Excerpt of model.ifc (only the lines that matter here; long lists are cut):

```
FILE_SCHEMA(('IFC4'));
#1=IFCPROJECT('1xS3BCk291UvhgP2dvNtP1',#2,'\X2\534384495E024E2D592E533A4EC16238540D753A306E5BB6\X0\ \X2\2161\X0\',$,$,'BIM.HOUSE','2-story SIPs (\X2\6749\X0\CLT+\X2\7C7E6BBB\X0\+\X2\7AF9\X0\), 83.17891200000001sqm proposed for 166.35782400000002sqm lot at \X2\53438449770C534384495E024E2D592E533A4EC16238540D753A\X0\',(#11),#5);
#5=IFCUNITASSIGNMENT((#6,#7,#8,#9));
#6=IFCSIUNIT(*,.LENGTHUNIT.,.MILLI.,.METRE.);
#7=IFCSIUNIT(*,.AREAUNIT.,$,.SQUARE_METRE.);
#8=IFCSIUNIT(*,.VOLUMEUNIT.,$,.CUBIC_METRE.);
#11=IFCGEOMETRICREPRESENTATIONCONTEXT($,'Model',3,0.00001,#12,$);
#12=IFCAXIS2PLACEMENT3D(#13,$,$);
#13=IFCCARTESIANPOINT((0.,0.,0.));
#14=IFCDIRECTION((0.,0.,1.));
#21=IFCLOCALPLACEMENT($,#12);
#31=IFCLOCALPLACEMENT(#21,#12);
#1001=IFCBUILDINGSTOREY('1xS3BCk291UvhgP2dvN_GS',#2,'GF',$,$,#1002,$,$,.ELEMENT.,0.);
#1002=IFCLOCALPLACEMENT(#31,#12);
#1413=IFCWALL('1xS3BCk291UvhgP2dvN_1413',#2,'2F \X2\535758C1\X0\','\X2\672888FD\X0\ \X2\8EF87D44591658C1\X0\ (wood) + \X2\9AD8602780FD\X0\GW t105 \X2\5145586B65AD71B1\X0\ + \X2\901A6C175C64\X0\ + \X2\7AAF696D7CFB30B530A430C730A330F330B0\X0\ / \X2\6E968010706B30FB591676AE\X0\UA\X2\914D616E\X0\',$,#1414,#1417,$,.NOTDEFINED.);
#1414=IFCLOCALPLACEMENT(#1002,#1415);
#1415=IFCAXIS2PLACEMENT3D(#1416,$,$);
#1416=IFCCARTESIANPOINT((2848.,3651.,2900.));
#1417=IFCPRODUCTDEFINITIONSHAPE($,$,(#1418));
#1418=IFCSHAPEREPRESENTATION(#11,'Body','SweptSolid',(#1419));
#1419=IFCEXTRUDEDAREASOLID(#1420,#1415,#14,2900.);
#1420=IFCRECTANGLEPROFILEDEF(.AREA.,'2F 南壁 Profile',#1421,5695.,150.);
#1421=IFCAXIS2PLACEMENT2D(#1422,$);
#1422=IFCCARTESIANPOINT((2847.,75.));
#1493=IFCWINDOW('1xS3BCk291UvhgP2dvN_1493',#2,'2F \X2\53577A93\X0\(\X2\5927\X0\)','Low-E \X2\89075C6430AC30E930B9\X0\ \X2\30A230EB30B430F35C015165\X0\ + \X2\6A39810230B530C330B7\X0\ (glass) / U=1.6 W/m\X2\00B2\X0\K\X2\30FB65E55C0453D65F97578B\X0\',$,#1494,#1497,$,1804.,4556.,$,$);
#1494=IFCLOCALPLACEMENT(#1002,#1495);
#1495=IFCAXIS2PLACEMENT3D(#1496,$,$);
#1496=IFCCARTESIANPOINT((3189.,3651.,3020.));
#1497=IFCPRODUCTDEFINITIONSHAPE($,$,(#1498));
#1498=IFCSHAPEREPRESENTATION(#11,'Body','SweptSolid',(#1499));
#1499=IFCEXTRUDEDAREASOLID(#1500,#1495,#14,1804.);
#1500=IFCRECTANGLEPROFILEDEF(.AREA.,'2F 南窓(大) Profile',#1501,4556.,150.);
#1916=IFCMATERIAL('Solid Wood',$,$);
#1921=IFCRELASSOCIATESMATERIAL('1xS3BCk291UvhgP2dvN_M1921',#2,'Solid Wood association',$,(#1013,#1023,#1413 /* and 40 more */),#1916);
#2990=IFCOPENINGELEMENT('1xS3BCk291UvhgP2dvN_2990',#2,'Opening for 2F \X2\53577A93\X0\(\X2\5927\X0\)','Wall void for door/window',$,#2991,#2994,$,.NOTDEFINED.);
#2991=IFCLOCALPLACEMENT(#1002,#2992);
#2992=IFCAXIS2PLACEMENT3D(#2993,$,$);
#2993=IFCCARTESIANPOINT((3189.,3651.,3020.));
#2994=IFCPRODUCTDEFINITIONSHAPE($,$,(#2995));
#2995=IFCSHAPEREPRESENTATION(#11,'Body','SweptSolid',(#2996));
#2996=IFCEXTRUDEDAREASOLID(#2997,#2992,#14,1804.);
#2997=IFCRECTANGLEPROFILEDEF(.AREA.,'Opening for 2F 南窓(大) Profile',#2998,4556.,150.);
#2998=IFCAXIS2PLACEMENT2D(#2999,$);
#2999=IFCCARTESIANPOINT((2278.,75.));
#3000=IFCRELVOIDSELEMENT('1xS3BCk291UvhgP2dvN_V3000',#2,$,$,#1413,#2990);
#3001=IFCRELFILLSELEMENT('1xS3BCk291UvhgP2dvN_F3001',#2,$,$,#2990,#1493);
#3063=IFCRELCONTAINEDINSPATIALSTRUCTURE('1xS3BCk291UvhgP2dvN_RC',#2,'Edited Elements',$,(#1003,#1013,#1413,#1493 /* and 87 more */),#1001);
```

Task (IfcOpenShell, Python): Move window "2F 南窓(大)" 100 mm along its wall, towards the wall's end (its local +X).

```python
import ifcopenshell
import ifcopenshell.api.geometry
import ifcopenshell.util.placement
import ifcopenshell.util.unit

model = ifcopenshell.open("model.ifc")
unit_scale = ifcopenshell.util.unit.calculate_unit_scale(model)

window = model.by_guid("1xS3BCk291UvhgP2dvN_1493")
opening = window.FillsVoids[0].RelatingOpeningElement
wall = opening.VoidsElements[0].RelatingBuildingElement

wall_matrix = ifcopenshell.util.placement.get_local_placement(wall.ObjectPlacement)
shift = wall_matrix[:3, 0] * 0.1 / unit_scale
before = ifcopenshell.util.placement.get_local_placement(window.ObjectPlacement)[:3, 3].copy()

# The window is not placed relative to its opening, so move both.
for product in (opening, window):
    matrix = ifcopenshell.util.placement.get_local_placement(product.ObjectPlacement)
    matrix[:3, 3] += shift
    ifcopenshell.api.geometry.edit_object_placement(model, product=product, matrix=matrix, is_si=False)

after = ifcopenshell.util.placement.get_local_placement(window.ObjectPlacement)[:3, 3]
print("window moved by", (after - before).round(3) + 0.0)

model.write("model-out.ifc")
```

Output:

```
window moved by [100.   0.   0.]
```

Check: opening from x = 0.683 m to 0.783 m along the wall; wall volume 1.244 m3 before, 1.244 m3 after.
